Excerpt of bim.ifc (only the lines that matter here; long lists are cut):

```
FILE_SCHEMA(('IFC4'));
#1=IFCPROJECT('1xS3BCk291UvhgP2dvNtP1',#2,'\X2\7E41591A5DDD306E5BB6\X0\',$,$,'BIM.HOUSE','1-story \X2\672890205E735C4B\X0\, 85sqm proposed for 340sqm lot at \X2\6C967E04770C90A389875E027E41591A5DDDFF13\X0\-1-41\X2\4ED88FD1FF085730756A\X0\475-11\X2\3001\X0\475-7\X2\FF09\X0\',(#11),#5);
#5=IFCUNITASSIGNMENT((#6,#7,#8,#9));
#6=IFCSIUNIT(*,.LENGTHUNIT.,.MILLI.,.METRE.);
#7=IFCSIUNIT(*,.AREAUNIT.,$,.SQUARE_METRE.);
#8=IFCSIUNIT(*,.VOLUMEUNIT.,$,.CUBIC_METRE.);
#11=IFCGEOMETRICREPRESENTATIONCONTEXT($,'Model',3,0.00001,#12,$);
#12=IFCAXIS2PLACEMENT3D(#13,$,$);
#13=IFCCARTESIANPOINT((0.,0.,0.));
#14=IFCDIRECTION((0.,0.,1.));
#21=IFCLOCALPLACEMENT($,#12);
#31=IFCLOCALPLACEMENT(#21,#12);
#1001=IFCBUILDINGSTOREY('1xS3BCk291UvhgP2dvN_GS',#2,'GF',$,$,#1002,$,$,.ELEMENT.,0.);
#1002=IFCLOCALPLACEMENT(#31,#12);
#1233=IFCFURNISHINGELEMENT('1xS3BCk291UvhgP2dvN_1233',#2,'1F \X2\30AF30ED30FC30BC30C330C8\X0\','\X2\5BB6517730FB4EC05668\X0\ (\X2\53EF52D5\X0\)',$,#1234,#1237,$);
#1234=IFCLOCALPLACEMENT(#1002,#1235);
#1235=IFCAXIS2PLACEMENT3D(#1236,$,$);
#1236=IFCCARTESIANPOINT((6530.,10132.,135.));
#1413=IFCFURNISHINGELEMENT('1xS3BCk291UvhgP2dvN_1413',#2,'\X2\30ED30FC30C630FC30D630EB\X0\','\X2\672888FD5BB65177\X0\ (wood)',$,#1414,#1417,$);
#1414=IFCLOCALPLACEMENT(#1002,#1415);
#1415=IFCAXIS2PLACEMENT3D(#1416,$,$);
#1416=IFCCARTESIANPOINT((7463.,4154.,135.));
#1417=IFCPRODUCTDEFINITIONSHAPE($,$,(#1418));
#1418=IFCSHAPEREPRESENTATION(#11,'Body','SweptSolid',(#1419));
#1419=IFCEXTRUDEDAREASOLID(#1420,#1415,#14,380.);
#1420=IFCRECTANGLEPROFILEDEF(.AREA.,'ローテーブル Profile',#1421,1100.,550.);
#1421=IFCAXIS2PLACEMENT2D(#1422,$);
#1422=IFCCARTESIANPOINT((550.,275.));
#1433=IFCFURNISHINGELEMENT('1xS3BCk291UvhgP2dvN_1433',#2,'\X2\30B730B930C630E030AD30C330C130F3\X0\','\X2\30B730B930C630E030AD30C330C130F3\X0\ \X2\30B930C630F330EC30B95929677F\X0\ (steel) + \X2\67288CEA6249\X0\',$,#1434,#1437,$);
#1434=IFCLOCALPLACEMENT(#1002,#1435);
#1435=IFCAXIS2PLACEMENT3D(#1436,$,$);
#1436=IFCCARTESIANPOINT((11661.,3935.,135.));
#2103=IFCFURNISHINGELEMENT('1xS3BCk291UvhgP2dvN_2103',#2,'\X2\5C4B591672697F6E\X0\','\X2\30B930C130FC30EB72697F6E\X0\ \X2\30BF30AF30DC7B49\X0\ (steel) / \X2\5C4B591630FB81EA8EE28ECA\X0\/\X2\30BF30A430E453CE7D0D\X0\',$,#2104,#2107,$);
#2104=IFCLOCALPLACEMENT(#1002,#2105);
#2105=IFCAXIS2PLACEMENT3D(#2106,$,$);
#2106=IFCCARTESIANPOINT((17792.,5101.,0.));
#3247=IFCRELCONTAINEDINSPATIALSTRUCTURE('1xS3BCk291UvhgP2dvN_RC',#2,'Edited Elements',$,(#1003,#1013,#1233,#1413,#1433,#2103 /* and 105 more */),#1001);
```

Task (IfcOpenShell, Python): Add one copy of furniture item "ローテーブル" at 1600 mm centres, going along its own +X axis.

```python
import ifcopenshell
import ifcopenshell.api.geometry
import ifcopenshell.api.root
import ifcopenshell.util.element
import ifcopenshell.util.placement
import ifcopenshell.util.unit

model = ifcopenshell.open("bim.ifc")
unit_scale = ifcopenshell.util.unit.calculate_unit_scale(model)


def reuse_history(source, copy):
    """copy_class also copies each property set's owner history, people and application; keep the originals."""
    for rel in copy.IsDefinedBy:
        if rel.is_a("IfcRelDefinesByProperties") and (history := rel.RelatingPropertyDefinition.OwnerHistory):
            rel.RelatingPropertyDefinition.OwnerHistory = source.OwnerHistory
            ifcopenshell.util.element.remove_deep2(model, history)


source = model.by_guid("1xS3BCk291UvhgP2dvN_1413")
base = ifcopenshell.util.placement.get_local_placement(source.ObjectPlacement)
step = base[:3, 0] * 1.6 / unit_scale

for i in range(1, 2):
    copy = ifcopenshell.api.root.copy_class(model, product=source)
    copy.Representation = ifcopenshell.util.element.copy_deep(
        model, source.Representation, exclude=["IfcGeometricRepresentationContext", "IfcRepresentationMap"]
    )
    reuse_history(source, copy)
    matrix = base.copy()
    matrix[:3, 3] += i * step
    print("added at", matrix[:3, 3].round(3) + 0.0)
    ifcopenshell.api.geometry.edit_object_placement(model, product=copy, matrix=matrix, is_si=False)

model.write("bim_rev.ifc")
```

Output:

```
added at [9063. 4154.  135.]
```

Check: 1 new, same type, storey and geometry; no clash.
